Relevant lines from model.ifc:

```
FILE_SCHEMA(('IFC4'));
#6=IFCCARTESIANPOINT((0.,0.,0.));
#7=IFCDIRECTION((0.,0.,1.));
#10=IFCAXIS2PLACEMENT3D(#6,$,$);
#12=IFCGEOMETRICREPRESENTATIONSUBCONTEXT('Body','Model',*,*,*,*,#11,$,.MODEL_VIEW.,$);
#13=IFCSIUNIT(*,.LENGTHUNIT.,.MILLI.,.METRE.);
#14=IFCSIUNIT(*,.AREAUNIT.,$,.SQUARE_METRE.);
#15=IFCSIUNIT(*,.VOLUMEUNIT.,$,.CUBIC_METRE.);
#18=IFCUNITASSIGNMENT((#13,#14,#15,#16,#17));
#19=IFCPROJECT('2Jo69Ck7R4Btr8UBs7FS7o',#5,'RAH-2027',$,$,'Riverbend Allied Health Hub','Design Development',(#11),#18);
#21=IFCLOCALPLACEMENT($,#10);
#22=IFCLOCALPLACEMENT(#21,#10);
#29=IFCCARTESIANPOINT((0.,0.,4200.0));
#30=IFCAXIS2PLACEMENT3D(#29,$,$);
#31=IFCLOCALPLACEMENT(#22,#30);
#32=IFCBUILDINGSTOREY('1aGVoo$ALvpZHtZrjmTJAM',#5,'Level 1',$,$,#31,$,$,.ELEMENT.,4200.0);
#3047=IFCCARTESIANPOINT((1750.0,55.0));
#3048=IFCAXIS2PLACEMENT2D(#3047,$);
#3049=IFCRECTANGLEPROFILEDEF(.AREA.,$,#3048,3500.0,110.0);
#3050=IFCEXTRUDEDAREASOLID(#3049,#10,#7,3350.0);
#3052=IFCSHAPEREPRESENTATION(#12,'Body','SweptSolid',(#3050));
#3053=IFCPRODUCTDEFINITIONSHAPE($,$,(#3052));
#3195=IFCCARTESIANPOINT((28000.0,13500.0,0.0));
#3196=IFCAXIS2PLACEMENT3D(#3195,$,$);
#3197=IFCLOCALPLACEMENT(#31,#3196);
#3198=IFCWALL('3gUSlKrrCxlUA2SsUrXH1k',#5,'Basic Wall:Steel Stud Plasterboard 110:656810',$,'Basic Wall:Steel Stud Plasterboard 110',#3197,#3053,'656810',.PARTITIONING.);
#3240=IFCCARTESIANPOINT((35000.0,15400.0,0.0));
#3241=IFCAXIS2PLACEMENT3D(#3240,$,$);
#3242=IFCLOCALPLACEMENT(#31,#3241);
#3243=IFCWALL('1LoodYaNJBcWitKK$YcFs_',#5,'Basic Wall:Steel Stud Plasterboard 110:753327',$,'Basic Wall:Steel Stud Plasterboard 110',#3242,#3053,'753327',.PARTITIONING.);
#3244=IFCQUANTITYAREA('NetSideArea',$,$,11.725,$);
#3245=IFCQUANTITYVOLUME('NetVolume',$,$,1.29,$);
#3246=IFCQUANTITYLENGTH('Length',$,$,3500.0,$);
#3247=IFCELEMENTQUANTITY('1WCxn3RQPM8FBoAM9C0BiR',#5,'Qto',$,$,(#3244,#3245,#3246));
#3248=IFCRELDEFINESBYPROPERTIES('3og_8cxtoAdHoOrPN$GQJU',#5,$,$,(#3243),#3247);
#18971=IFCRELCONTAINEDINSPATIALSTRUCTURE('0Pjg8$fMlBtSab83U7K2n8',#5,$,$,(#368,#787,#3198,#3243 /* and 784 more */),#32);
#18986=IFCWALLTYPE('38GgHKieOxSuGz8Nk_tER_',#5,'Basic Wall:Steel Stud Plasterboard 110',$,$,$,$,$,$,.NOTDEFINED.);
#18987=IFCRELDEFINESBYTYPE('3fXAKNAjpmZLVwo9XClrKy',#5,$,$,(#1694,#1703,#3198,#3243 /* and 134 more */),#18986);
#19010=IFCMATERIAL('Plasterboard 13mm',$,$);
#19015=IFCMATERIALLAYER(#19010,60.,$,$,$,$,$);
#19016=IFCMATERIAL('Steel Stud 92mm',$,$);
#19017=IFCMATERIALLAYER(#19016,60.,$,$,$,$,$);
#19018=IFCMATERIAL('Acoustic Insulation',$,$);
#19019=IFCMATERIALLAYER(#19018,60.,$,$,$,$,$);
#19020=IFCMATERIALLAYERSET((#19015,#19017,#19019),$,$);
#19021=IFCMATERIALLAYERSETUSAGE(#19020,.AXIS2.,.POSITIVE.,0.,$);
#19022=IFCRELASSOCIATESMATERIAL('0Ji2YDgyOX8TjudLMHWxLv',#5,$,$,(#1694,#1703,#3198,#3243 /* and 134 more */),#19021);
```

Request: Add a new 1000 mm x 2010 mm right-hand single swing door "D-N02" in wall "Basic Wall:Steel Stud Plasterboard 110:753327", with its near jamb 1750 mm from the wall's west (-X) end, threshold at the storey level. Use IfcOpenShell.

```python
import numpy as np
import ifcopenshell
import ifcopenshell.api.feature
import ifcopenshell.api.geometry
import ifcopenshell.api.pset
import ifcopenshell.api.root
import ifcopenshell.api.spatial
import ifcopenshell.geom
import ifcopenshell.util.element
import ifcopenshell.util.placement
import ifcopenshell.util.representation
import ifcopenshell.util.shape
import ifcopenshell.util.unit

model = ifcopenshell.open("model.ifc")
unit_scale = ifcopenshell.util.unit.calculate_unit_scale(model)
area_scale = ifcopenshell.util.unit.calculate_unit_scale(model, "AREAUNIT")
volume_scale = ifcopenshell.util.unit.calculate_unit_scale(model, "VOLUMEUNIT")
settings = ifcopenshell.geom.settings()


def volume(element):
    """Net volume in cubic metres, openings subtracted."""
    shape = ifcopenshell.geom.create_shape(settings, element)
    return ifcopenshell.util.shape.get_volume(shape.geometry)


wall = model.by_id(3243)
storey = ifcopenshell.util.element.get_container(wall, ifc_class="IfcBuildingStorey")
context = ifcopenshell.util.representation.get_context(model, "Model", "Body", "MODEL_VIEW")
before = volume(wall)

width, height, from_end, sill = 1, 2.01, 1.75, 0.0  # metres

# The wall runs along its own X axis, and the end named is its -X end.
wall_shape = ifcopenshell.geom.create_shape(settings, wall)
x, y, z = ifcopenshell.util.shape.get_vertices(wall_shape.geometry).T
start = x.min() + from_end
face, thickness = float(y.min()), float(y.max() - y.min())
wall_matrix = ifcopenshell.util.placement.get_local_placement(wall.ObjectPlacement)
level = ifcopenshell.util.placement.get_local_placement(storey.ObjectPlacement)[2, 3]


def in_wall(x, y):
    """Placement at x, y metres in the wall's axes, at sill height."""
    matrix = wall_matrix.copy()
    matrix[:, 3] = wall_matrix @ np.array([x / unit_scale, y / unit_scale, 0.0, 1.0])
    matrix[2, 3] = level + sill / unit_scale
    return matrix


# Opening: a box that overshoots both wall faces by 50 mm.
opening = ifcopenshell.api.root.create_entity(model, ifc_class="IfcOpeningElement", predefined_type="OPENING")
box = ifcopenshell.api.geometry.add_wall_representation(
    model, context=context, length=width, height=height, thickness=thickness + 0.1
)
ifcopenshell.api.geometry.assign_representation(model, product=opening, representation=box)
ifcopenshell.api.geometry.edit_object_placement(model, product=opening, matrix=in_wall(start, face - 0.05), is_si=False)
ifcopenshell.api.feature.add_feature(model, feature=opening, element=wall)

door = ifcopenshell.api.root.create_entity(model, ifc_class="IfcDoor", name="D-N02", predefined_type="DOOR")
door.OverallWidth, door.OverallHeight = width / unit_scale, height / unit_scale
door.OperationType = "SINGLE_SWING_RIGHT"
body = ifcopenshell.api.geometry.add_door_representation(
    model,
    context=context,
    overall_width=door.OverallWidth,
    overall_height=door.OverallHeight,
    operation_type="SINGLE_SWING_RIGHT",
    lining_properties={"LiningDepth": thickness / unit_scale, "ThresholdDepth": thickness / unit_scale},
)
ifcopenshell.api.geometry.assign_representation(model, product=door, representation=body)
ifcopenshell.api.spatial.assign_container(model, products=[door], relating_structure=storey)
ifcopenshell.api.feature.add_filling(model, opening=opening, element=door)

# The lining spans the wall, so the door starts at the wall face.
ifcopenshell.api.geometry.edit_object_placement(model, product=door, matrix=in_wall(start, face), is_si=False)

after = volume(wall)

# Update the wall's stored quantities.
qto = model.by_id(ifcopenshell.util.element.get_pset(wall, "Qto", should_inherit=False)["id"])
ifcopenshell.api.pset.edit_qto(model, qto=qto, properties={
    "NetSideArea": after / thickness / area_scale,
    "NetVolume": after / volume_scale,
})

print(f"wall volume {before:.3f} -> {after:.3f} m3")

model.write("model_v2.ifc")
```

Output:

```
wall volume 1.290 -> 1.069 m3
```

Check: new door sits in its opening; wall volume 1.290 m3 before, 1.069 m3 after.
